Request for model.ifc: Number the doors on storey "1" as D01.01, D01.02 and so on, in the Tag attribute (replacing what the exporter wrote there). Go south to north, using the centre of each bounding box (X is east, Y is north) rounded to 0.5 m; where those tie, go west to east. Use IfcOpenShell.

First a look at what the model holds.

```python
import ifcopenshell
import ifcopenshell.util.element
import ifcopenshell.util.placement

model = ifcopenshell.open("model.ifc")
print(model.schema)
storey = next(s for s in model.by_type("IfcBuildingStorey") if s.Name == "1")
doors = [e for e in ifcopenshell.util.element.get_decomposition(storey) if e.is_a("IfcDoor")]
for e in sorted(doors, key=lambda e: e.id()):
    origin = ifcopenshell.util.placement.get_local_placement(e.ObjectPlacement)[:3, 3]
    print(e.id(), e.Tag, e.Name, origin.round(2) + 0.0, sep=" | ")
```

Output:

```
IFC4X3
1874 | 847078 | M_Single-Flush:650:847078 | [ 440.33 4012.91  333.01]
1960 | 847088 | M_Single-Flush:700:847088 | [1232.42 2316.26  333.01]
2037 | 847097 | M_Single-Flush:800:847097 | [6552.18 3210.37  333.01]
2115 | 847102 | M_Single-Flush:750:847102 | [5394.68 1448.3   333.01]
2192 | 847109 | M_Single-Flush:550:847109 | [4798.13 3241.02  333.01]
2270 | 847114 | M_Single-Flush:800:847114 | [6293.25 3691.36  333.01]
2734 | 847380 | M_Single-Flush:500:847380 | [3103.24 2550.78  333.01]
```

```python
import ifcopenshell
import ifcopenshell.geom
import ifcopenshell.util.element
import ifcopenshell.util.shape

model = ifcopenshell.open("model.ifc")
settings = ifcopenshell.geom.settings()
settings.set("use-world-coords", True)


def centre(element):
    shape = ifcopenshell.geom.create_shape(settings, element)
    return ifcopenshell.util.shape.get_bbox_centroid(shape.geometry)


storey = next(s for s in model.by_type("IfcBuildingStorey") if s.Name == "1")
doors = [e for e in ifcopenshell.util.element.get_decomposition(storey) if e.is_a("IfcDoor")]

# Insertion points can sit at a corner or the storey origin, so sort by the geometry (in metres).
centres = {e: centre(e) for e in doors}
doors.sort(key=lambda e: (round(centres[e][1] / 0.5), centres[e][0]))

for i, e in enumerate(doors, start=1):
    number = f"D01.{i:02d}"
    e.Tag = number
    print(e.id(), number)

model.write("model_rev.ifc")
```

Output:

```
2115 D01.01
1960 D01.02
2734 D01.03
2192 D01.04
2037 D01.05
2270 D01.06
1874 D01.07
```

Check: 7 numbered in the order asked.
